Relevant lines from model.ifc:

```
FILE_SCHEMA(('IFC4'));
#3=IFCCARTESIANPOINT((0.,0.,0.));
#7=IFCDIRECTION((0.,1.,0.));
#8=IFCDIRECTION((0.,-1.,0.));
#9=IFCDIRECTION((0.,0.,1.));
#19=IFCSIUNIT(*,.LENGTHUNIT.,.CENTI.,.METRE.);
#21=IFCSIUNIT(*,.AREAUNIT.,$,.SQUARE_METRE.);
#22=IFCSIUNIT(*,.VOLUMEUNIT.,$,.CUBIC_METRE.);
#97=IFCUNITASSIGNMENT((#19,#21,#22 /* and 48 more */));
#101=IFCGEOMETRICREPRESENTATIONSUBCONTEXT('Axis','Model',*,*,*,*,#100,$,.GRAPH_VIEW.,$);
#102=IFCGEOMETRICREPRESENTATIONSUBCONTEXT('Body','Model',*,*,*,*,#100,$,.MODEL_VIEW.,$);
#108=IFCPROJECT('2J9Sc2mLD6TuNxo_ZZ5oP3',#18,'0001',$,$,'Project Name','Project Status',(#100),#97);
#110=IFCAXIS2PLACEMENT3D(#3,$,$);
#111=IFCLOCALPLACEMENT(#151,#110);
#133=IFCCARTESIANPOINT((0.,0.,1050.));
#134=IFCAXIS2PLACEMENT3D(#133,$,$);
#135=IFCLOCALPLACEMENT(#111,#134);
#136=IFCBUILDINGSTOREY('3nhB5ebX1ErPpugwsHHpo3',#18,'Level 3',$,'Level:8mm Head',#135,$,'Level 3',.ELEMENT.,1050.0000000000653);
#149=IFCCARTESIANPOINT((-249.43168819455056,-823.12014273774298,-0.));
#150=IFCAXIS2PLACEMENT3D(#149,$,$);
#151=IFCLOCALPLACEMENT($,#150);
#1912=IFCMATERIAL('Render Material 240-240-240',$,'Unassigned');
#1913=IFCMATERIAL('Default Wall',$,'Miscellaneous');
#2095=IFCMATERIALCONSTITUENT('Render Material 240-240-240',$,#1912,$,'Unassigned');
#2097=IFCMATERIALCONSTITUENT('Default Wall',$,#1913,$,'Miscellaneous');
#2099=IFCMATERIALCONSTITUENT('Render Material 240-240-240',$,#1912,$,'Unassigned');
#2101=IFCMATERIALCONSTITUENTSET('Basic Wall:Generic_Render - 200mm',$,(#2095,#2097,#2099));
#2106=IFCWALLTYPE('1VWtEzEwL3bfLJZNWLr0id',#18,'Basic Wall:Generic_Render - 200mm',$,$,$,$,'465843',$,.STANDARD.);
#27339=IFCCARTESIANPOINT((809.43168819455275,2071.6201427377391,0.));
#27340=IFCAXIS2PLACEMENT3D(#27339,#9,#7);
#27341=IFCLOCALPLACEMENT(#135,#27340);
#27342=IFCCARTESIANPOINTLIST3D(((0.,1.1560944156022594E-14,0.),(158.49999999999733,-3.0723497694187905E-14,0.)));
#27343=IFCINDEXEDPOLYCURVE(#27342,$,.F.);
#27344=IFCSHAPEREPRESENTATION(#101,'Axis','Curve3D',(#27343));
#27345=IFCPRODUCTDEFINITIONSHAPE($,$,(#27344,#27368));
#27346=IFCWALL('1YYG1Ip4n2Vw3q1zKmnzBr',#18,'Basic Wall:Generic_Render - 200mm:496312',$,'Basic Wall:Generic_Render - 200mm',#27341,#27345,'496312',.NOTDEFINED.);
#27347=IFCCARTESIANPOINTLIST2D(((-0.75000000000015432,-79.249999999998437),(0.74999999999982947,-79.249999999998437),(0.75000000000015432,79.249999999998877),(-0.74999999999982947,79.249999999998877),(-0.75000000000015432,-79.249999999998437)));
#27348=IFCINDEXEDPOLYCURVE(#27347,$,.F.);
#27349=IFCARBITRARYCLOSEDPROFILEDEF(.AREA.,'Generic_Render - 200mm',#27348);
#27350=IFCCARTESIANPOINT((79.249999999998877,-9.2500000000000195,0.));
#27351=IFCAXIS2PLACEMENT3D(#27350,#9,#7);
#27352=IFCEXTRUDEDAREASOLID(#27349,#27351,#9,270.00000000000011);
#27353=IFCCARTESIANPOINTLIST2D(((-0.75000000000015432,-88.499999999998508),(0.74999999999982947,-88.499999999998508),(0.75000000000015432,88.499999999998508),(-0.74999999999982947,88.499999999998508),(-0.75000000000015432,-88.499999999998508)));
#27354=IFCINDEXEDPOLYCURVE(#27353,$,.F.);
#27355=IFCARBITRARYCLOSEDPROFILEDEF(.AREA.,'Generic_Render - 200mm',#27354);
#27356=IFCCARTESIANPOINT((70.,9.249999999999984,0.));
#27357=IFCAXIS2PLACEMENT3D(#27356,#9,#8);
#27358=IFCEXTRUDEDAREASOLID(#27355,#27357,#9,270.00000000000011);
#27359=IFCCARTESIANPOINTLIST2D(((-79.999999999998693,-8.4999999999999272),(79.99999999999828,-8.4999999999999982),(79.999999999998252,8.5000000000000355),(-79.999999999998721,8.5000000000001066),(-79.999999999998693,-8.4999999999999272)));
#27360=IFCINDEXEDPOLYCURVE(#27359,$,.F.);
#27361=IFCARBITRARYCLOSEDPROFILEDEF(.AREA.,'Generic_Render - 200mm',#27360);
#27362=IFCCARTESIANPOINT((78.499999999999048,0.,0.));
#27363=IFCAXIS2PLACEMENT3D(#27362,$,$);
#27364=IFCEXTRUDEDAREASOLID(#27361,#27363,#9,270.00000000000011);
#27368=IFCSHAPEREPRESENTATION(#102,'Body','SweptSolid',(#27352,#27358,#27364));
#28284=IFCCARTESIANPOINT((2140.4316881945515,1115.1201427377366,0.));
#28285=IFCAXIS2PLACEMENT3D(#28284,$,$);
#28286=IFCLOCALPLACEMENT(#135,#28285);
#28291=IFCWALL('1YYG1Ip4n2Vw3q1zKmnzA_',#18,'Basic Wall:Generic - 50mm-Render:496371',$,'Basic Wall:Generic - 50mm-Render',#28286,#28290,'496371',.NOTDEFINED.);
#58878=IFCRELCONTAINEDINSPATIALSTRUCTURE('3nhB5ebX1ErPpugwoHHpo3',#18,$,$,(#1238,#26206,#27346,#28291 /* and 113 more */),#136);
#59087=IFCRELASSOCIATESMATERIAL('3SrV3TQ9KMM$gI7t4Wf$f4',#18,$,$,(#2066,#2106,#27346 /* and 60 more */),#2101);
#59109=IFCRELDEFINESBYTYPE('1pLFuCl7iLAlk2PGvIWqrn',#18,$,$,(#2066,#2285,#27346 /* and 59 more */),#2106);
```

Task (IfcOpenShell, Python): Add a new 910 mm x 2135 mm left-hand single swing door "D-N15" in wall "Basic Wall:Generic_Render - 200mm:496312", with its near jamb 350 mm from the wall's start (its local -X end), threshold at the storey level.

```python
import numpy as np
import ifcopenshell
import ifcopenshell.api.feature
import ifcopenshell.api.geometry
import ifcopenshell.api.root
import ifcopenshell.api.spatial
import ifcopenshell.geom
import ifcopenshell.util.element
import ifcopenshell.util.placement
import ifcopenshell.util.representation
import ifcopenshell.util.shape
import ifcopenshell.util.unit

model = ifcopenshell.open("model.ifc")
unit_scale = ifcopenshell.util.unit.calculate_unit_scale(model)
settings = ifcopenshell.geom.settings()


def volume(element):
    """Net volume in cubic metres, openings subtracted."""
    shape = ifcopenshell.geom.create_shape(settings, element)
    return ifcopenshell.util.shape.get_volume(shape.geometry)


wall = model.by_guid("1YYG1Ip4n2Vw3q1zKmnzBr")
storey = ifcopenshell.util.element.get_container(wall, ifc_class="IfcBuildingStorey")
context = ifcopenshell.util.representation.get_context(model, "Model", "Body", "MODEL_VIEW")
before = volume(wall)

width, height, from_end, sill = 0.91, 2.135, 0.35, 0.0  # metres

# The wall runs along its own X axis, and the end named is its -X end.
wall_shape = ifcopenshell.geom.create_shape(settings, wall)
x, y, z = ifcopenshell.util.shape.get_vertices(wall_shape.geometry).T
start = x.min() + from_end
face, thickness = float(y.min()), float(y.max() - y.min())
wall_matrix = ifcopenshell.util.placement.get_local_placement(wall.ObjectPlacement)
level = ifcopenshell.util.placement.get_local_placement(storey.ObjectPlacement)[2, 3]


def in_wall(x, y):
    """Placement at x, y metres in the wall's axes, at sill height."""
    matrix = wall_matrix.copy()
    matrix[:, 3] = wall_matrix @ np.array([x / unit_scale, y / unit_scale, 0.0, 1.0])
    matrix[2, 3] = level + sill / unit_scale
    return matrix


# Opening: a box that overshoots both wall faces by 50 mm.
opening = ifcopenshell.api.root.create_entity(model, ifc_class="IfcOpeningElement", predefined_type="OPENING")
box = ifcopenshell.api.geometry.add_wall_representation(
    model, context=context, length=width, height=height, thickness=thickness + 0.1
)
ifcopenshell.api.geometry.assign_representation(model, product=opening, representation=box)
ifcopenshell.api.geometry.edit_object_placement(model, product=opening, matrix=in_wall(start, face - 0.05), is_si=False)
ifcopenshell.api.feature.add_feature(model, feature=opening, element=wall)

door = ifcopenshell.api.root.create_entity(model, ifc_class="IfcDoor", name="D-N15", predefined_type="DOOR")
door.OverallWidth, door.OverallHeight = width / unit_scale, height / unit_scale
door.OperationType = "SINGLE_SWING_LEFT"
body = ifcopenshell.api.geometry.add_door_representation(
    model,
    context=context,
    overall_width=door.OverallWidth,
    overall_height=door.OverallHeight,
    operation_type="SINGLE_SWING_LEFT",
    lining_properties={"LiningDepth": thickness / unit_scale, "ThresholdDepth": thickness / unit_scale},
)
ifcopenshell.api.geometry.assign_representation(model, product=door, representation=body)
ifcopenshell.api.spatial.assign_container(model, products=[door], relating_structure=storey)
ifcopenshell.api.feature.add_filling(model, opening=opening, element=door)

# The lining spans the wall, so the door starts at the wall face.
ifcopenshell.api.geometry.edit_object_placement(model, product=door, matrix=in_wall(start, face), is_si=False)

after = volume(wall)

print(f"wall volume {before:.3f} -> {after:.3f} m3")

model.write("model_updated.ifc")
```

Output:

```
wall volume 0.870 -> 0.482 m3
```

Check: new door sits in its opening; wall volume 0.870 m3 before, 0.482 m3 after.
